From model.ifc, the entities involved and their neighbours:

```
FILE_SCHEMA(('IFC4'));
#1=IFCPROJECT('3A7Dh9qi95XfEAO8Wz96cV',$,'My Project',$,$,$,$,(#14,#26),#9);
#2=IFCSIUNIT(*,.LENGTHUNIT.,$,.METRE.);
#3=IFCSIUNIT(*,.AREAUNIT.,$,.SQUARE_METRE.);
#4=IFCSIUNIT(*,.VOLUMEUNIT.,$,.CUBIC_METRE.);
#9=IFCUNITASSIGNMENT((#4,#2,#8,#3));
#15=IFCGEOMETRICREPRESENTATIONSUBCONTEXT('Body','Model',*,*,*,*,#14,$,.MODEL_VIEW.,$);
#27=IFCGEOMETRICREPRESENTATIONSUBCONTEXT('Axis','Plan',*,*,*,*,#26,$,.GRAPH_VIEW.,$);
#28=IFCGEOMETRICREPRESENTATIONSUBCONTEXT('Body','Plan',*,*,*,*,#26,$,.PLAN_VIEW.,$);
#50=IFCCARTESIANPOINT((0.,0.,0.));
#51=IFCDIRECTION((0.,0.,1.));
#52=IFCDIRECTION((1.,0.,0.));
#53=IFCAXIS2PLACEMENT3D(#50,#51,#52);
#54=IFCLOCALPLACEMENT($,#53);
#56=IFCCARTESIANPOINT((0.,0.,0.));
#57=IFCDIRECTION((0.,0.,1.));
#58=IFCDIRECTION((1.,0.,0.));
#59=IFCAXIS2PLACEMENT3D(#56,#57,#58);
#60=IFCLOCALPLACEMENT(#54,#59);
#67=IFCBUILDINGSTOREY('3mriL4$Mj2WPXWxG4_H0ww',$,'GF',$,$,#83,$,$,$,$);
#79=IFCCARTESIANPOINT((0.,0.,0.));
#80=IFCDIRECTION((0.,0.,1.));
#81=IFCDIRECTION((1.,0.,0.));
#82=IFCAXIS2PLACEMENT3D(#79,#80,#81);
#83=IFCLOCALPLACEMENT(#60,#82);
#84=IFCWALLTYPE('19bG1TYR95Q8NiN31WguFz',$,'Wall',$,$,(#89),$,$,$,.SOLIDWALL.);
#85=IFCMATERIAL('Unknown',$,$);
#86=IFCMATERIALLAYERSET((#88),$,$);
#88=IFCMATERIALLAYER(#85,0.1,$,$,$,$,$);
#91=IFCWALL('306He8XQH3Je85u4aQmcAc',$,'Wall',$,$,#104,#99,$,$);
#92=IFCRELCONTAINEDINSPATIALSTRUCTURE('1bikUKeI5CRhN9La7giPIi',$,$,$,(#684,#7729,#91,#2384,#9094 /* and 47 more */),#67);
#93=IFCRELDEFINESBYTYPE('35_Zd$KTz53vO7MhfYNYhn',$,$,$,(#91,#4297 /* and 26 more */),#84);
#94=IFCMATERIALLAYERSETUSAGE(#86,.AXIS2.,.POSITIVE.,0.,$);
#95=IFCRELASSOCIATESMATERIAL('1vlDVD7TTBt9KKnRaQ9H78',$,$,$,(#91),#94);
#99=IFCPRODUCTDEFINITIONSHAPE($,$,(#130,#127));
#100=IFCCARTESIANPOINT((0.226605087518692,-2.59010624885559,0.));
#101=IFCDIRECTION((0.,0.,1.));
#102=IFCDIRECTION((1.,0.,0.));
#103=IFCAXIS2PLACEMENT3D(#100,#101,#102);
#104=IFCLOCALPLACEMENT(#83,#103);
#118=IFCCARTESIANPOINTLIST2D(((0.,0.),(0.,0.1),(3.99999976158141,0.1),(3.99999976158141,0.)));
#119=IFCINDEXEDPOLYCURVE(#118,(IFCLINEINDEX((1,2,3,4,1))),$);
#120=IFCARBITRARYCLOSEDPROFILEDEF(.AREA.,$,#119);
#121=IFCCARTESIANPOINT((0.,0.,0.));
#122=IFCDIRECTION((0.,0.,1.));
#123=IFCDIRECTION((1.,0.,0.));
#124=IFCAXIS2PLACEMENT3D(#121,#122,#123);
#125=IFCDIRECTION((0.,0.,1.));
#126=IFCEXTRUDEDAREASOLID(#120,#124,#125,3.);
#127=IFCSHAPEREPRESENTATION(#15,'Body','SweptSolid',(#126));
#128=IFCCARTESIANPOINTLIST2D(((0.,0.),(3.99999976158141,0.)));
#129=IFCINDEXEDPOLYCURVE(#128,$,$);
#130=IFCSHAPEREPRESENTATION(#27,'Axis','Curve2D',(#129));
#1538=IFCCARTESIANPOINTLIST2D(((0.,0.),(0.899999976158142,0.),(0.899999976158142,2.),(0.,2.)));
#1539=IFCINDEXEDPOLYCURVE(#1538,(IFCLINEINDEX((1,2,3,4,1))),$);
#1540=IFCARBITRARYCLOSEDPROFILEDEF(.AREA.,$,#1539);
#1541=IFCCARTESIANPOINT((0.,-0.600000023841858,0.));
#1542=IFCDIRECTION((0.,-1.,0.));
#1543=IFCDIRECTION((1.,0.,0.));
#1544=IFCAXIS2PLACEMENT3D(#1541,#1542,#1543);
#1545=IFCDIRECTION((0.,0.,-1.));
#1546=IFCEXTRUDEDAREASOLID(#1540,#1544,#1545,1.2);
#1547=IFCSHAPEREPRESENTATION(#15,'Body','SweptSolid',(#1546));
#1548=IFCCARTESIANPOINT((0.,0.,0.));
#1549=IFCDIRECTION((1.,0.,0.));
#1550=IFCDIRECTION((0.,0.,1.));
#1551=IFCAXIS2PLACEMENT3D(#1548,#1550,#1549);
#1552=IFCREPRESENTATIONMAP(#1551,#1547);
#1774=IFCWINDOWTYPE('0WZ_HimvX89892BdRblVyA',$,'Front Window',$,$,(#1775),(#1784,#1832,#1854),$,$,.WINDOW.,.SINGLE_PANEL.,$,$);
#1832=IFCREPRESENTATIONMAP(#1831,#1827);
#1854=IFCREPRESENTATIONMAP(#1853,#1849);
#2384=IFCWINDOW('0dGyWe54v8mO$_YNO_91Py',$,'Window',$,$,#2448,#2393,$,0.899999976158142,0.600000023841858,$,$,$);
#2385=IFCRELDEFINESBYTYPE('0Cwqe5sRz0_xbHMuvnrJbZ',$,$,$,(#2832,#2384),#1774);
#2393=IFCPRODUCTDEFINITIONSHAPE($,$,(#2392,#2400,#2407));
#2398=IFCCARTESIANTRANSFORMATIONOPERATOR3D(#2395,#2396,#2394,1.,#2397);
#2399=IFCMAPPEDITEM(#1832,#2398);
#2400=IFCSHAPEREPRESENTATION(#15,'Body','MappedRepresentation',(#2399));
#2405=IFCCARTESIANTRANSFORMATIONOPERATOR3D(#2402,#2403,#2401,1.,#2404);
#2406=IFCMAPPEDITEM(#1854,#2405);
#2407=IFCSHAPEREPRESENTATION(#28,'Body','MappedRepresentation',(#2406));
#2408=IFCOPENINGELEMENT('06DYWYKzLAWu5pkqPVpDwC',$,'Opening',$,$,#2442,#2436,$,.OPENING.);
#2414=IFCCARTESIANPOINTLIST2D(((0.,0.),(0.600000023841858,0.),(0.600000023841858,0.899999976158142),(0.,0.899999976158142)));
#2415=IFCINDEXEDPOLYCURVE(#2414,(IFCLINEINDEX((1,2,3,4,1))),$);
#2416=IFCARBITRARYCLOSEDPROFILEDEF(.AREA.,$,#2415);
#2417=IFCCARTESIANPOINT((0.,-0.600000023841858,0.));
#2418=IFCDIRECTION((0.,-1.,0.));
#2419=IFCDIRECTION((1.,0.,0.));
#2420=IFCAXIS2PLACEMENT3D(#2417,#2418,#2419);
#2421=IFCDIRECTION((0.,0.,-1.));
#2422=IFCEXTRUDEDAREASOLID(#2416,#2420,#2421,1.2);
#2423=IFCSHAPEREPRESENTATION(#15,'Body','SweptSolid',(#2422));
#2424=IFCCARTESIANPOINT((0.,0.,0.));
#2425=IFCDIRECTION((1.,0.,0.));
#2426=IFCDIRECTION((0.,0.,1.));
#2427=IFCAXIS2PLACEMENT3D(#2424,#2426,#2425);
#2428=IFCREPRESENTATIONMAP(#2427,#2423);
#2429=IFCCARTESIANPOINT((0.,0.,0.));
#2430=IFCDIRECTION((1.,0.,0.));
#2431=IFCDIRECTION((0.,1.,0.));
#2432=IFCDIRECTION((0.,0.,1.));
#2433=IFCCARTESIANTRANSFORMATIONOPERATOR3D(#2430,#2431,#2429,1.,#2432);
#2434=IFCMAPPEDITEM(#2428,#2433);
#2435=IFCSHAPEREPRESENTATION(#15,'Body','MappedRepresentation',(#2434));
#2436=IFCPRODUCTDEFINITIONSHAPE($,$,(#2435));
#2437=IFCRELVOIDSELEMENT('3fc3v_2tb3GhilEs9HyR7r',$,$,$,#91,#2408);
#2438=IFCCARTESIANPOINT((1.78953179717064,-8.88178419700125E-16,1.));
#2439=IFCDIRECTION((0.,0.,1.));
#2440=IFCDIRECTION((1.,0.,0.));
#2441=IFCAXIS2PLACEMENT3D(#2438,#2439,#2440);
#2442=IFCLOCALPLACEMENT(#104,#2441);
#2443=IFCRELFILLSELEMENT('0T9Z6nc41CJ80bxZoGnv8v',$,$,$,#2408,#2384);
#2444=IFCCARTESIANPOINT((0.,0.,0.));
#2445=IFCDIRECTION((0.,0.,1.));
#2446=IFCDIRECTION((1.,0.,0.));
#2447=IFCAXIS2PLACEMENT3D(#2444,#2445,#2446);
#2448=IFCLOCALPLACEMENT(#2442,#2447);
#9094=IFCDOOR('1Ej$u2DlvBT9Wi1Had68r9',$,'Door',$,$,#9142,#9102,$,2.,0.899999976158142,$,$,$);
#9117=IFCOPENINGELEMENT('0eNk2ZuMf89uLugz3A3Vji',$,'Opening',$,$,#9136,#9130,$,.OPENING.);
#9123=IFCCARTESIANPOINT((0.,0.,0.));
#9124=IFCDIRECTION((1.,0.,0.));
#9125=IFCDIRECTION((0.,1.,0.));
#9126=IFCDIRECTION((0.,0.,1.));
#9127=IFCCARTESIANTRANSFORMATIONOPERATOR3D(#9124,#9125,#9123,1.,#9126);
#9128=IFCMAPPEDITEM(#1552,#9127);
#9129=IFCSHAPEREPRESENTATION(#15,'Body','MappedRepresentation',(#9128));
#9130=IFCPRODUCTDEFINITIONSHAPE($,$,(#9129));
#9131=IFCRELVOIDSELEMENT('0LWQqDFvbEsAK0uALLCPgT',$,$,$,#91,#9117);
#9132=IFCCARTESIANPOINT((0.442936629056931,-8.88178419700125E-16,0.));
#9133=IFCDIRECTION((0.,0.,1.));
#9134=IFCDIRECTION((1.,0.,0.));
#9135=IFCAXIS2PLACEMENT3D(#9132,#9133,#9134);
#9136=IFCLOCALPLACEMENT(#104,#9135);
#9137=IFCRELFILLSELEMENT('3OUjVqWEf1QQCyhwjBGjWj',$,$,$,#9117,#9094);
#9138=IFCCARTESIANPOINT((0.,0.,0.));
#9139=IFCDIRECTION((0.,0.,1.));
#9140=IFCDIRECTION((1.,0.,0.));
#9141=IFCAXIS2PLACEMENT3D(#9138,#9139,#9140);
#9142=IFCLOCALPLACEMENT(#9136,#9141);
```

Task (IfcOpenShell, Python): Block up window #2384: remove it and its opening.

```python
import ifcopenshell
import ifcopenshell.api.feature
import ifcopenshell.api.root
import ifcopenshell.geom
import ifcopenshell.util.shape

model = ifcopenshell.open("model.ifc")
settings = ifcopenshell.geom.settings()


def volume(element):
    """Net volume in cubic metres, openings subtracted."""
    shape = ifcopenshell.geom.create_shape(settings, element)
    return ifcopenshell.util.shape.get_volume(shape.geometry)


window = model.by_id(2384)
opening = window.FillsVoids[0].RelatingOpeningElement
wall = opening.VoidsElements[0].RelatingBuildingElement
before = volume(wall)

ifcopenshell.api.root.remove_product(model, product=window)
ifcopenshell.api.feature.remove_feature(model, feature=opening)

after = volume(wall)

print(f"wall volume {before:.3f} -> {after:.3f} m3")

model.write("model_v2.ifc")
```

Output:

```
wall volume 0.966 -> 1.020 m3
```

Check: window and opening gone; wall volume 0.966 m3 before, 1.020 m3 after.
